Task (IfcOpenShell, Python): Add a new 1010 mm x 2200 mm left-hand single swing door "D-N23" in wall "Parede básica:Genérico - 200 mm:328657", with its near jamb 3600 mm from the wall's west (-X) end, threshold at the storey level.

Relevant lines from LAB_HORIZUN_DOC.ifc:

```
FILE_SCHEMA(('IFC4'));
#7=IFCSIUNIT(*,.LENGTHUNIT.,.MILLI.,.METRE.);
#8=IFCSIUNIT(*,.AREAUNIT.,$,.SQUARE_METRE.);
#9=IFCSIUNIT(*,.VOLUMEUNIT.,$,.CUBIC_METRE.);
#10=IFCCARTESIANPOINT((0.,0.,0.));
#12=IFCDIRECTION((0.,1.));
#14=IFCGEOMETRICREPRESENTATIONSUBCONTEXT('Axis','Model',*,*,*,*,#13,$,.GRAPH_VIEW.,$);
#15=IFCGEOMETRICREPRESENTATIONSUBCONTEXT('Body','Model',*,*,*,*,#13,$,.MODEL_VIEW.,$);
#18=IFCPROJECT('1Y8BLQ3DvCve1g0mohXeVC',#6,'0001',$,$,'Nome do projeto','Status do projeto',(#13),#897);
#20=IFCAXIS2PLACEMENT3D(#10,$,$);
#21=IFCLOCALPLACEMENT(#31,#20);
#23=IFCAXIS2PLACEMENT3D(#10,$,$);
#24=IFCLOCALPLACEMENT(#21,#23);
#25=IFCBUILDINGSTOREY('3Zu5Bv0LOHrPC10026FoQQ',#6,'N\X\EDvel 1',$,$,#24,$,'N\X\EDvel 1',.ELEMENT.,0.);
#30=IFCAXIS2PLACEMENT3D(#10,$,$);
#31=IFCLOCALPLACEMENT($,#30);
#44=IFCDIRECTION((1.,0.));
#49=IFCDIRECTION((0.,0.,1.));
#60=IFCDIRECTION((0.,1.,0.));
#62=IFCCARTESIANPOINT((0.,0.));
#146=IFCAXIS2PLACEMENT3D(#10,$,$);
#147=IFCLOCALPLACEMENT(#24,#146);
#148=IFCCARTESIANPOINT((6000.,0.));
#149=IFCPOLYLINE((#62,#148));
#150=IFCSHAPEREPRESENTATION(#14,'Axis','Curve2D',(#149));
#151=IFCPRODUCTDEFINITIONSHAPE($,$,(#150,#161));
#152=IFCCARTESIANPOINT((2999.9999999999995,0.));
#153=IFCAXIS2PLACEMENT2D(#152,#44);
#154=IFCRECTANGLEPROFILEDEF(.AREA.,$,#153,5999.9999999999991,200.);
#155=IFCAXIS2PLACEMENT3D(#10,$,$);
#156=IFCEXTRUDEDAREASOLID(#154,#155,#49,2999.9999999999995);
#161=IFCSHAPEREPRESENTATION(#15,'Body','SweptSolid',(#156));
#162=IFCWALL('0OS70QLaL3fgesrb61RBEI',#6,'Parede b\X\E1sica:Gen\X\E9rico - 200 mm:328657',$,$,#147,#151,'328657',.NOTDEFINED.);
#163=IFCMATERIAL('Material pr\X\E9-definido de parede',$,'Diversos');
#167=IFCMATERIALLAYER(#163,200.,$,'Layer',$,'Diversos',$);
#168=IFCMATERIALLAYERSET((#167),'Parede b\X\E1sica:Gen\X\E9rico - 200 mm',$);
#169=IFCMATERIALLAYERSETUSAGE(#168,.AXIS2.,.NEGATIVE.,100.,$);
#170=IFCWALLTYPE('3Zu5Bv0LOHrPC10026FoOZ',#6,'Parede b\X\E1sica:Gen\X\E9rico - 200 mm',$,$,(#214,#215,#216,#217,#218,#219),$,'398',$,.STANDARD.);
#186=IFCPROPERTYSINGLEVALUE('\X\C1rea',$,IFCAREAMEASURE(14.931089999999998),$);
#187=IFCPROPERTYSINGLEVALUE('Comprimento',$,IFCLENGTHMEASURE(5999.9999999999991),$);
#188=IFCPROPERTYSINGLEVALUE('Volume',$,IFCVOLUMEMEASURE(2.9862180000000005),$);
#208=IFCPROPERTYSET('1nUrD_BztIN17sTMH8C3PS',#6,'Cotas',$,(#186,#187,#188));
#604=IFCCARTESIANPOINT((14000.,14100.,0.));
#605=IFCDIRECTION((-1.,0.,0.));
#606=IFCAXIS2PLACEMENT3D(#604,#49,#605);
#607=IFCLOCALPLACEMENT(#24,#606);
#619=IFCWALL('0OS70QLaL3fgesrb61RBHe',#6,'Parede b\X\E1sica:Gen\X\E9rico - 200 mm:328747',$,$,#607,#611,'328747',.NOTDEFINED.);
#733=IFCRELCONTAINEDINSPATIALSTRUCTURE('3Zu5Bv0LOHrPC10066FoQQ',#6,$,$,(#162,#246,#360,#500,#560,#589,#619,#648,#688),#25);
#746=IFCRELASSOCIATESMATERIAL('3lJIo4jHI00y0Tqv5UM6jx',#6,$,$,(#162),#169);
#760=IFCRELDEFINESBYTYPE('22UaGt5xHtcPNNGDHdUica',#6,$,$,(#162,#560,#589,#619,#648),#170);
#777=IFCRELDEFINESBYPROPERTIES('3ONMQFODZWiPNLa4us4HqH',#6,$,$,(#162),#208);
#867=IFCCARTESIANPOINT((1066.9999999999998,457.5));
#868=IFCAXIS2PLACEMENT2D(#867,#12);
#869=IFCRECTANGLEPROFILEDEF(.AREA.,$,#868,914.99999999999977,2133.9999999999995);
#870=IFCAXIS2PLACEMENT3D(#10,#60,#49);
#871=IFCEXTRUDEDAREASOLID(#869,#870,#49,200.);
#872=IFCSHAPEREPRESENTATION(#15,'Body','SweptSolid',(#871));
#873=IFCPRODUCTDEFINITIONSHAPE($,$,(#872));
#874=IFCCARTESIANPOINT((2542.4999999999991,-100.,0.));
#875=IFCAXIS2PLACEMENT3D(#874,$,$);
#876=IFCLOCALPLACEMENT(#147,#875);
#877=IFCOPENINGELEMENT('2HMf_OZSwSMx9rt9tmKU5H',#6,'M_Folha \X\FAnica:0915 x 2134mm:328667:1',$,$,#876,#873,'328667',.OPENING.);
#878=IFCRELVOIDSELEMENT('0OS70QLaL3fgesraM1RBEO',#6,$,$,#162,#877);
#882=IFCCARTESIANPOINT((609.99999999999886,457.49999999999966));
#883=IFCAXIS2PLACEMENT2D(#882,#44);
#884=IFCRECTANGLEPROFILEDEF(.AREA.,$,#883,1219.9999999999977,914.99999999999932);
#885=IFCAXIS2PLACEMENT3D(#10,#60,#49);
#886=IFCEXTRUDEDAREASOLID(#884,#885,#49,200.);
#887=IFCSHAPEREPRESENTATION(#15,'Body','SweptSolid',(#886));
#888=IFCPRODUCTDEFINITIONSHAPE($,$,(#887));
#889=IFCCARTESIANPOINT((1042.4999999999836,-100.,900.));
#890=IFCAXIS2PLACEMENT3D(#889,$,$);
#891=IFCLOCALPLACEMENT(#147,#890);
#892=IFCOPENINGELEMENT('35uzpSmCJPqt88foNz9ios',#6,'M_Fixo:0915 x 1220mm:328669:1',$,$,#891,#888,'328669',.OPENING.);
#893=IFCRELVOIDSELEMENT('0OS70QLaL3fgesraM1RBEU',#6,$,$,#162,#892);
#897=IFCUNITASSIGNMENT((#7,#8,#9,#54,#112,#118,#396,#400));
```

```python
import numpy as np
import ifcopenshell
import ifcopenshell.api.feature
import ifcopenshell.api.geometry
import ifcopenshell.api.pset
import ifcopenshell.api.root
import ifcopenshell.api.spatial
import ifcopenshell.geom
import ifcopenshell.util.element
import ifcopenshell.util.placement
import ifcopenshell.util.representation
import ifcopenshell.util.shape
import ifcopenshell.util.unit

model = ifcopenshell.open("LAB_HORIZUN_DOC.ifc")
unit_scale = ifcopenshell.util.unit.calculate_unit_scale(model)
area_scale = ifcopenshell.util.unit.calculate_unit_scale(model, "AREAUNIT")
volume_scale = ifcopenshell.util.unit.calculate_unit_scale(model, "VOLUMEUNIT")
settings = ifcopenshell.geom.settings()


def volume(element):
    """Net volume in cubic metres, openings subtracted."""
    shape = ifcopenshell.geom.create_shape(settings, element)
    return ifcopenshell.util.shape.get_volume(shape.geometry)


wall = model.by_id(162)
storey = ifcopenshell.util.element.get_container(wall, ifc_class="IfcBuildingStorey")
context = ifcopenshell.util.representation.get_context(model, "Model", "Body", "MODEL_VIEW")
before = volume(wall)

width, height, from_end, sill = 1.01, 2.2, 3.6, 0.0  # metres

# The wall runs along its own X axis, and the end named is its -X end.
wall_shape = ifcopenshell.geom.create_shape(settings, wall)
x, y, z = ifcopenshell.util.shape.get_vertices(wall_shape.geometry).T
start = x.min() + from_end
face, thickness = float(y.min()), float(y.max() - y.min())
wall_matrix = ifcopenshell.util.placement.get_local_placement(wall.ObjectPlacement)
level = ifcopenshell.util.placement.get_local_placement(storey.ObjectPlacement)[2, 3]


def in_wall(x, y):
    """Placement at x, y metres in the wall's axes, at sill height."""
    matrix = wall_matrix.copy()
    matrix[:, 3] = wall_matrix @ np.array([x / unit_scale, y / unit_scale, 0.0, 1.0])
    matrix[2, 3] = level + sill / unit_scale
    return matrix


# Opening: a box that overshoots both wall faces by 50 mm.
opening = ifcopenshell.api.root.create_entity(model, ifc_class="IfcOpeningElement", predefined_type="OPENING")
box = ifcopenshell.api.geometry.add_wall_representation(
    model, context=context, length=width, height=height, thickness=thickness + 0.1
)
ifcopenshell.api.geometry.assign_representation(model, product=opening, representation=box)
ifcopenshell.api.geometry.edit_object_placement(model, product=opening, matrix=in_wall(start, face - 0.05), is_si=False)
ifcopenshell.api.feature.add_feature(model, feature=opening, element=wall)

door = ifcopenshell.api.root.create_entity(model, ifc_class="IfcDoor", name="D-N23", predefined_type="DOOR")
door.OverallWidth, door.OverallHeight = width / unit_scale, height / unit_scale
door.OperationType = "SINGLE_SWING_LEFT"
body = ifcopenshell.api.geometry.add_door_representation(
    model,
    context=context,
    overall_width=door.OverallWidth,
    overall_height=door.OverallHeight,
    operation_type="SINGLE_SWING_LEFT",
    lining_properties={"LiningDepth": thickness / unit_scale, "ThresholdDepth": thickness / unit_scale},
)
ifcopenshell.api.geometry.assign_representation(model, product=door, representation=body)
ifcopenshell.api.spatial.assign_container(model, products=[door], relating_structure=storey)
ifcopenshell.api.feature.add_filling(model, opening=opening, element=door)

# The lining spans the wall, so the door starts at the wall face.
ifcopenshell.api.geometry.edit_object_placement(model, product=door, matrix=in_wall(start, face), is_si=False)

after = volume(wall)

# Update the wall's stored quantities.
pset = model.by_id(ifcopenshell.util.element.get_pset(wall, "Cotas", should_inherit=False)["id"])
ifcopenshell.api.pset.edit_pset(model, pset=pset, properties={
    "Área": model.create_entity("IfcAreaMeasure", after / thickness / area_scale),
    "Volume": model.create_entity("IfcVolumeMeasure", after / volume_scale),
})

print(f"wall volume {before:.3f} -> {after:.3f} m3")

model.write("LAB_HORIZUN_DOC_edited.ifc")
```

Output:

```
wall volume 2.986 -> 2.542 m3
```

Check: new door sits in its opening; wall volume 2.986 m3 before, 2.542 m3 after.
